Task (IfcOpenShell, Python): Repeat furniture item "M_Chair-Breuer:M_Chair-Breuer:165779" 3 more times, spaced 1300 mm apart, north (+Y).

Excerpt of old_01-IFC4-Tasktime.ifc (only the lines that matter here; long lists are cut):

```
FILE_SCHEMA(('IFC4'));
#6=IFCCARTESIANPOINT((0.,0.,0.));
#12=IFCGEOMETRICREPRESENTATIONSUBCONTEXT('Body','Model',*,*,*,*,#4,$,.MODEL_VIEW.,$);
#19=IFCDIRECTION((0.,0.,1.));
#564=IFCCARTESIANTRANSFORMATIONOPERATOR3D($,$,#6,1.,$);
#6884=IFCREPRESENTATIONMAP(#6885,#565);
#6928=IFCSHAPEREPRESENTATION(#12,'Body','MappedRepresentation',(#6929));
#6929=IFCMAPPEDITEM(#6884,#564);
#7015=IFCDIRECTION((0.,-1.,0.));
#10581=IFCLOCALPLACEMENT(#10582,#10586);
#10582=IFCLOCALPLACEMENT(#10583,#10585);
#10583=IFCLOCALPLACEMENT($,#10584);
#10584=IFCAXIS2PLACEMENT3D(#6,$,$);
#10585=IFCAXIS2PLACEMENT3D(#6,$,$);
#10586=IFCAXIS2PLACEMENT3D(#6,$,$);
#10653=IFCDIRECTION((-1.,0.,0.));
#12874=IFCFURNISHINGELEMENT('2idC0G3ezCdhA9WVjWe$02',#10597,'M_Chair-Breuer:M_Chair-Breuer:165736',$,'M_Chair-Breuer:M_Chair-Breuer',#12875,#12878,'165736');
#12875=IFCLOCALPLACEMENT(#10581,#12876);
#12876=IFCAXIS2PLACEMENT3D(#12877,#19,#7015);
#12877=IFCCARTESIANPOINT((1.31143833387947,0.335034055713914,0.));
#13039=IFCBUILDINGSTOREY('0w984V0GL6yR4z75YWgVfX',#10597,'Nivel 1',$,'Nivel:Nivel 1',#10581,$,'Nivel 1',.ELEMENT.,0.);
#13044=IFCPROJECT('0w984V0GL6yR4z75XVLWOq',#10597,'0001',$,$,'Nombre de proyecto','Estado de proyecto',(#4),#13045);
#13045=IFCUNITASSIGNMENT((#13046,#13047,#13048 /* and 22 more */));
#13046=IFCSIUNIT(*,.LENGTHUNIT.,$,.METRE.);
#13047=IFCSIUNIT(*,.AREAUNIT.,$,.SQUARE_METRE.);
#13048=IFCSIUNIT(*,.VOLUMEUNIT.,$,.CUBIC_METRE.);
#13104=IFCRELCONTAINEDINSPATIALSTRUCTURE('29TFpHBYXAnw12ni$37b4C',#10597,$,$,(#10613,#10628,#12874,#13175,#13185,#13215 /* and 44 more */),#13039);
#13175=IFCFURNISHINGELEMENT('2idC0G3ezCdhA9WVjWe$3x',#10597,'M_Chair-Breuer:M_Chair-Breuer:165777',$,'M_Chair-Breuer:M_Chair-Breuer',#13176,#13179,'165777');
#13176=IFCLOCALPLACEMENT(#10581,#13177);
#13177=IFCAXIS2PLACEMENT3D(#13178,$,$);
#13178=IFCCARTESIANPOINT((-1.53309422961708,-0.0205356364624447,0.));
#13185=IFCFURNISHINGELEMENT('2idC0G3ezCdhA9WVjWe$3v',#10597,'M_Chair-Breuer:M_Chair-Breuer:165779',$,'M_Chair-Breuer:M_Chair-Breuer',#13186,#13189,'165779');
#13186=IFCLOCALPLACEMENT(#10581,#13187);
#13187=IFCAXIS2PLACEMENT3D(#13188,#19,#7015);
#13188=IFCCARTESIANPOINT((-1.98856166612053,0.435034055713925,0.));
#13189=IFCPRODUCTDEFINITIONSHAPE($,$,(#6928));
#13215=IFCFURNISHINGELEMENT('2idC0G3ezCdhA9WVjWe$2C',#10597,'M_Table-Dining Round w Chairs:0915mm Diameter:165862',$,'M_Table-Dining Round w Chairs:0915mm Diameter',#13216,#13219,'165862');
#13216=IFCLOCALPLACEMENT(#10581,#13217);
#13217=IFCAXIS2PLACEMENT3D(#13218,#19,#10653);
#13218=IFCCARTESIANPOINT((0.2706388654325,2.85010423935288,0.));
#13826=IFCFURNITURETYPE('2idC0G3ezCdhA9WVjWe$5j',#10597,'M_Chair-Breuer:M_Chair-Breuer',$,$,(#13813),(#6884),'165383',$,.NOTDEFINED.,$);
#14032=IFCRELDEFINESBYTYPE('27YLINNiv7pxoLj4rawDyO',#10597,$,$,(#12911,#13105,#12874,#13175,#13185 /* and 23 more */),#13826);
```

```python
import numpy as np
import ifcopenshell
import ifcopenshell.api.geometry
import ifcopenshell.api.root
import ifcopenshell.util.element
import ifcopenshell.util.placement
import ifcopenshell.util.unit

model = ifcopenshell.open("old_01-IFC4-Tasktime.ifc")
unit_scale = ifcopenshell.util.unit.calculate_unit_scale(model)


def reuse_history(source, copy):
    """copy_class also copies each property set's owner history, people and application; keep the originals."""
    for rel in copy.IsDefinedBy:
        if rel.is_a("IfcRelDefinesByProperties") and (history := rel.RelatingPropertyDefinition.OwnerHistory):
            rel.RelatingPropertyDefinition.OwnerHistory = source.OwnerHistory
            ifcopenshell.util.element.remove_deep2(model, history)


source = model.by_guid("2idC0G3ezCdhA9WVjWe$3v")
base = ifcopenshell.util.placement.get_local_placement(source.ObjectPlacement)
step = np.array([0.0, 1.0, 0.0]) * 1.3 / unit_scale

for i in range(1, 4):
    copy = ifcopenshell.api.root.copy_class(model, product=source)
    copy.Representation = ifcopenshell.util.element.copy_deep(
        model, source.Representation, exclude=["IfcGeometricRepresentationContext", "IfcRepresentationMap"]
    )
    copy.Name = "M_Chair-Breuer:M_Chair-Breuer"
    copy.Tag = None
    reuse_history(source, copy)
    matrix = base.copy()
    matrix[:3, 3] += i * step
    print("added at", matrix[:3, 3].round(3) + 0.0)
    ifcopenshell.api.geometry.edit_object_placement(model, product=copy, matrix=matrix, is_si=False)

model.write("old_01-IFC4-Tasktime_edited.ifc")
```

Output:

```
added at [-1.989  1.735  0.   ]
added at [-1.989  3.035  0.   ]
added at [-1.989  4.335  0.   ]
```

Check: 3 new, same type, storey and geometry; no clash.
